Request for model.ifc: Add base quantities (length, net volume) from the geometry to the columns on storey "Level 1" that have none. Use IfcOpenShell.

First a look at what the model holds.

```python
import ifcopenshell
import ifcopenshell.util.element
import ifcopenshell.util.unit

model = ifcopenshell.open("model.ifc")
print(model.schema)
for unit_type in ("LENGTHUNIT", "AREAUNIT", "VOLUMEUNIT"):
    print(unit_type, ifcopenshell.util.unit.calculate_unit_scale(model, unit_type))
storey = next(s for s in model.by_type("IfcBuildingStorey") if s.Name == "Level 1")
columns = [e for e in ifcopenshell.util.element.get_decomposition(storey) if e.is_a("IfcColumn")]
for e in sorted(columns, key=lambda e: e.id()):
    print(e.id(), e.is_a(), e.Name, list(ifcopenshell.util.element.get_psets(e, qtos_only=True)), sep=" | ")
```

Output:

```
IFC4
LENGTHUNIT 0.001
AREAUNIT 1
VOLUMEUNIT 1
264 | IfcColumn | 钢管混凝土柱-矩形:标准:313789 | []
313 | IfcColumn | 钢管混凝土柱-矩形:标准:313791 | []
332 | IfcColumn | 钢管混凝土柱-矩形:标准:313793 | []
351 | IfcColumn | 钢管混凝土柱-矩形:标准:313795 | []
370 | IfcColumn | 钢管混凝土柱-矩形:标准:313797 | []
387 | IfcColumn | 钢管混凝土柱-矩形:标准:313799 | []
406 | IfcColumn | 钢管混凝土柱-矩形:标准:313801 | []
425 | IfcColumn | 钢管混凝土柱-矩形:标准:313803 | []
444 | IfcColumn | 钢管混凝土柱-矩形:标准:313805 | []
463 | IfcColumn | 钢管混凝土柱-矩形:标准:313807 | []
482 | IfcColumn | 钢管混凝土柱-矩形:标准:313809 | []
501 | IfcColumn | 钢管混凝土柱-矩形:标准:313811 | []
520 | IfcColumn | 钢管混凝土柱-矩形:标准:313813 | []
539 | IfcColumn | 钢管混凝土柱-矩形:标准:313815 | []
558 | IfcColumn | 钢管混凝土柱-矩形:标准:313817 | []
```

```python
import ifcopenshell
import ifcopenshell.api.pset
import ifcopenshell.geom
import ifcopenshell.util.element
import ifcopenshell.util.shape
import ifcopenshell.util.unit

model = ifcopenshell.open("model.ifc")
unit_scale = ifcopenshell.util.unit.calculate_unit_scale(model)
volume_scale = ifcopenshell.util.unit.calculate_unit_scale(model, "VOLUMEUNIT")
settings = ifcopenshell.geom.settings()

storey = next(s for s in model.by_type("IfcBuildingStorey") if s.Name == "Level 1")
columns = [e for e in ifcopenshell.util.element.get_decomposition(storey) if e.is_a("IfcColumn")]

for e in sorted(columns, key=lambda e: e.id()):
    if ifcopenshell.util.element.get_psets(e, qtos_only=True, should_inherit=False):
        continue
    # Geometry comes back in metres, in the element's own axes.
    shape = ifcopenshell.geom.create_shape(settings, e)
    values = {
        "Length": ifcopenshell.util.shape.get_z(shape.geometry) / unit_scale,
        "NetVolume": ifcopenshell.util.shape.get_volume(shape.geometry) / volume_scale,
    }
    qto = ifcopenshell.api.pset.add_qto(model, product=e, name="Qto_ColumnBaseQuantities")
    ifcopenshell.api.pset.edit_qto(model, qto=qto, properties=values)
    print(e.id(), {k: round(v, 3) for k, v in values.items()})

model.write("model_updated.ifc")
```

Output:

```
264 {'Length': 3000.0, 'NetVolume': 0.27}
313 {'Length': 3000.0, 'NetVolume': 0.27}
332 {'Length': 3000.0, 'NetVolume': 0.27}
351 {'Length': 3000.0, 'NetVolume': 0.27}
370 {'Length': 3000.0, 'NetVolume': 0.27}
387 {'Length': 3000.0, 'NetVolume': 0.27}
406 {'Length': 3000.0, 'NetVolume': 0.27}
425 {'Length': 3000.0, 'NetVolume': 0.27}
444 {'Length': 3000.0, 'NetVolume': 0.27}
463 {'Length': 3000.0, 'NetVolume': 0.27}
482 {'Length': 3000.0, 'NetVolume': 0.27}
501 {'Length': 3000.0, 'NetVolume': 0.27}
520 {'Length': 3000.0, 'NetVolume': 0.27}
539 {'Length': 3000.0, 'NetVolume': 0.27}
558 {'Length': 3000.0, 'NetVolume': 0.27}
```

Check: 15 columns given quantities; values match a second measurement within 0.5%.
